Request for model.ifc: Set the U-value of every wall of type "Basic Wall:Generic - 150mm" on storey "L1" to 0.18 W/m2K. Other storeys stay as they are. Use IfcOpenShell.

First a look at what the model holds.

```python
import ifcopenshell
import ifcopenshell.util.element

model = ifcopenshell.open("model.ifc")
print(model.schema)
storey = next(s for s in model.by_type("IfcBuildingStorey") if s.Name == "L1")
walls = [e for e in ifcopenshell.util.element.get_decomposition(storey) if e.is_a("IfcWall")]
seen = {}
for e in walls:
    element_type = ifcopenshell.util.element.get_type(e)
    key = (element_type.Name if element_type != e and element_type else None, ifcopenshell.util.element.get_pset(e, "Pset_WallCommon", "ThermalTransmittance"))
    seen[key] = seen.get(key, 0) + 1
for (name, value), count in sorted(seen.items(), key=str):
    print(count, "x", name, "|", value)
```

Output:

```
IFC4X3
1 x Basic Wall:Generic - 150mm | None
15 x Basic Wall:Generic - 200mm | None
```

```python
import ifcopenshell
import ifcopenshell.api.pset
import ifcopenshell.util.element

model = ifcopenshell.open("model.ifc")

storey = next(s for s in model.by_type("IfcBuildingStorey") if s.Name == "L1")
walls = [e for e in ifcopenshell.util.element.get_decomposition(storey) if e.is_a("IfcWall")]

count = 0
for e in walls:
    element_type = ifcopenshell.util.element.get_type(e)
    if element_type in (None, e) or element_type.Name != "Basic Wall:Generic - 150mm":
        continue
    # add_pset returns the element's existing set when there is one.
    pset = ifcopenshell.api.pset.add_pset(model, product=e, name="Pset_WallCommon")
    ifcopenshell.api.pset.edit_pset(model, pset=pset, properties={"ThermalTransmittance": 0.18})
    count += 1

print(count, "walls updated")

model.write("model_updated.ifc")
```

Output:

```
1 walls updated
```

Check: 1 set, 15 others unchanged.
